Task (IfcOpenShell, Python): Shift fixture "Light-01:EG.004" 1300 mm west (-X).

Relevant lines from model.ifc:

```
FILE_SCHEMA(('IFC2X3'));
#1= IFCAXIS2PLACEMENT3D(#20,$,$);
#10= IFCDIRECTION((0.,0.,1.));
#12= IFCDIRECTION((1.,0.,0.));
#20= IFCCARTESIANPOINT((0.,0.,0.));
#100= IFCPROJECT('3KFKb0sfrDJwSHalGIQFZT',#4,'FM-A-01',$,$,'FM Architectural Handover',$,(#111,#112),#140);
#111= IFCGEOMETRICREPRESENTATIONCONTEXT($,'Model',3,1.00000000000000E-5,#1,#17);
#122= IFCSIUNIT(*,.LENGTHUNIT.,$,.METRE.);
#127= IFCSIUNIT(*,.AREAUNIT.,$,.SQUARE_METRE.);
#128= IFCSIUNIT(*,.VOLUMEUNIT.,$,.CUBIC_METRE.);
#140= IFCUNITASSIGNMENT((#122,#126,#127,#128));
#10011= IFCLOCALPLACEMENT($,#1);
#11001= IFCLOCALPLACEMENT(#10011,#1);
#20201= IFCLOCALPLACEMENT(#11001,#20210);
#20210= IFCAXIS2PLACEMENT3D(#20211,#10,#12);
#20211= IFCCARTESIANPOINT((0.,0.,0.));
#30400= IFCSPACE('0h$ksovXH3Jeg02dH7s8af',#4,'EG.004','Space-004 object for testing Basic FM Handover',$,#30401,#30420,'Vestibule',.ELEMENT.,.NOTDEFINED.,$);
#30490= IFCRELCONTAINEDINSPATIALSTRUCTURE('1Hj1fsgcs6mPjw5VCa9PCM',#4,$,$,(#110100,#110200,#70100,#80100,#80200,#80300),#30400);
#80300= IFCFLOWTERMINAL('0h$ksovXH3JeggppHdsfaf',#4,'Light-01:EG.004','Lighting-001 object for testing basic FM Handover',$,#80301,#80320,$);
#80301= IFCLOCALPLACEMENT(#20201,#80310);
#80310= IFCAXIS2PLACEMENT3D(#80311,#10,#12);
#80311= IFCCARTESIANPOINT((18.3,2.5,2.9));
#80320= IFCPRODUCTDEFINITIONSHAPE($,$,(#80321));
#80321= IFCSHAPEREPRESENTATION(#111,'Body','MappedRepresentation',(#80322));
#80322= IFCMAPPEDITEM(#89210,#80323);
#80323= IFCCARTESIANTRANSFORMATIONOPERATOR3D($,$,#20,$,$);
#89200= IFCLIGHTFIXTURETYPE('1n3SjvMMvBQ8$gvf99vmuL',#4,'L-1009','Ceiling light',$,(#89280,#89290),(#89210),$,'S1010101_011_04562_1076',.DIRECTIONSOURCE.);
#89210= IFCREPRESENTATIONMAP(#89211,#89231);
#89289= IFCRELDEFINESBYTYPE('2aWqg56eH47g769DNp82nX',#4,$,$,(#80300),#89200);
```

```python
import ifcopenshell
import ifcopenshell.api.geometry
import ifcopenshell.util.placement
import ifcopenshell.util.unit

model = ifcopenshell.open("model.ifc")
unit_scale = ifcopenshell.util.unit.calculate_unit_scale(model)

item = model.by_guid("0h$ksovXH3JeggppHdsfaf")
matrix = ifcopenshell.util.placement.get_local_placement(item.ObjectPlacement)
matrix[0, 3] -= 1.3 / unit_scale
ifcopenshell.api.geometry.edit_object_placement(model, product=item, matrix=matrix, is_si=False)

print(ifcopenshell.util.placement.get_local_placement(item.ObjectPlacement).round(3) + 0.0)

model.write("model-out.ifc")
```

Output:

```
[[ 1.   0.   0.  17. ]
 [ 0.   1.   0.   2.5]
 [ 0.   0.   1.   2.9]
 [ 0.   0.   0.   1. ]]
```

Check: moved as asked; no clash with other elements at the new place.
